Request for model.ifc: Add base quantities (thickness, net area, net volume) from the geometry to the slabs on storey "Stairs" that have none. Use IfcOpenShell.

First a look at what the model holds.

```python
import ifcopenshell
import ifcopenshell.util.element
import ifcopenshell.util.unit

model = ifcopenshell.open("model.ifc")
print(model.schema)
for unit_type in ("LENGTHUNIT", "AREAUNIT", "VOLUMEUNIT"):
    print(unit_type, ifcopenshell.util.unit.calculate_unit_scale(model, unit_type))
storey = next(s for s in model.by_type("IfcBuildingStorey") if s.Name == "Stairs")
slabs = [e for e in ifcopenshell.util.element.get_decomposition(storey) if e.is_a("IfcSlab")]
for e in sorted(slabs, key=lambda e: e.id()):
    print(e.id(), e.is_a(), e.Name, list(ifcopenshell.util.element.get_psets(e, qtos_only=True)), sep=" | ")
```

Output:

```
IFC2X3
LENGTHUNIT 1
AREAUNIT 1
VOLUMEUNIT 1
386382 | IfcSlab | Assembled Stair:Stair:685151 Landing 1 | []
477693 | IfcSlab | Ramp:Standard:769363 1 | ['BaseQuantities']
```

```python
import ifcopenshell
import ifcopenshell.api.pset
import ifcopenshell.geom
import ifcopenshell.util.element
import ifcopenshell.util.shape
import ifcopenshell.util.unit

model = ifcopenshell.open("model.ifc")
unit_scale = ifcopenshell.util.unit.calculate_unit_scale(model)
area_scale = ifcopenshell.util.unit.calculate_unit_scale(model, "AREAUNIT")
volume_scale = ifcopenshell.util.unit.calculate_unit_scale(model, "VOLUMEUNIT")
settings = ifcopenshell.geom.settings()

storey = next(s for s in model.by_type("IfcBuildingStorey") if s.Name == "Stairs")
slabs = [e for e in ifcopenshell.util.element.get_decomposition(storey) if e.is_a("IfcSlab")]

for e in sorted(slabs, key=lambda e: e.id()):
    if ifcopenshell.util.element.get_psets(e, qtos_only=True, should_inherit=False):
        continue
    # Geometry comes back in metres, in the element's own axes.
    shape = ifcopenshell.geom.create_shape(settings, e)
    values = {
        "Width": ifcopenshell.util.shape.get_z(shape.geometry) / unit_scale,
        "NetArea": ifcopenshell.util.shape.get_footprint_area(shape.geometry) / area_scale,
        "NetVolume": ifcopenshell.util.shape.get_volume(shape.geometry) / volume_scale,
    }
    qto = ifcopenshell.api.pset.add_qto(model, product=e, name="BaseQuantities")
    ifcopenshell.api.pset.edit_qto(model, qto=qto, properties=values)
    print(e.id(), {k: round(v, 3) for k, v in values.items()})

model.write("model_edited.ifc")
```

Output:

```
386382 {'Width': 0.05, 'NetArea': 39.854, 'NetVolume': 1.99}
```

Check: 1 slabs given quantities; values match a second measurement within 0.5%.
